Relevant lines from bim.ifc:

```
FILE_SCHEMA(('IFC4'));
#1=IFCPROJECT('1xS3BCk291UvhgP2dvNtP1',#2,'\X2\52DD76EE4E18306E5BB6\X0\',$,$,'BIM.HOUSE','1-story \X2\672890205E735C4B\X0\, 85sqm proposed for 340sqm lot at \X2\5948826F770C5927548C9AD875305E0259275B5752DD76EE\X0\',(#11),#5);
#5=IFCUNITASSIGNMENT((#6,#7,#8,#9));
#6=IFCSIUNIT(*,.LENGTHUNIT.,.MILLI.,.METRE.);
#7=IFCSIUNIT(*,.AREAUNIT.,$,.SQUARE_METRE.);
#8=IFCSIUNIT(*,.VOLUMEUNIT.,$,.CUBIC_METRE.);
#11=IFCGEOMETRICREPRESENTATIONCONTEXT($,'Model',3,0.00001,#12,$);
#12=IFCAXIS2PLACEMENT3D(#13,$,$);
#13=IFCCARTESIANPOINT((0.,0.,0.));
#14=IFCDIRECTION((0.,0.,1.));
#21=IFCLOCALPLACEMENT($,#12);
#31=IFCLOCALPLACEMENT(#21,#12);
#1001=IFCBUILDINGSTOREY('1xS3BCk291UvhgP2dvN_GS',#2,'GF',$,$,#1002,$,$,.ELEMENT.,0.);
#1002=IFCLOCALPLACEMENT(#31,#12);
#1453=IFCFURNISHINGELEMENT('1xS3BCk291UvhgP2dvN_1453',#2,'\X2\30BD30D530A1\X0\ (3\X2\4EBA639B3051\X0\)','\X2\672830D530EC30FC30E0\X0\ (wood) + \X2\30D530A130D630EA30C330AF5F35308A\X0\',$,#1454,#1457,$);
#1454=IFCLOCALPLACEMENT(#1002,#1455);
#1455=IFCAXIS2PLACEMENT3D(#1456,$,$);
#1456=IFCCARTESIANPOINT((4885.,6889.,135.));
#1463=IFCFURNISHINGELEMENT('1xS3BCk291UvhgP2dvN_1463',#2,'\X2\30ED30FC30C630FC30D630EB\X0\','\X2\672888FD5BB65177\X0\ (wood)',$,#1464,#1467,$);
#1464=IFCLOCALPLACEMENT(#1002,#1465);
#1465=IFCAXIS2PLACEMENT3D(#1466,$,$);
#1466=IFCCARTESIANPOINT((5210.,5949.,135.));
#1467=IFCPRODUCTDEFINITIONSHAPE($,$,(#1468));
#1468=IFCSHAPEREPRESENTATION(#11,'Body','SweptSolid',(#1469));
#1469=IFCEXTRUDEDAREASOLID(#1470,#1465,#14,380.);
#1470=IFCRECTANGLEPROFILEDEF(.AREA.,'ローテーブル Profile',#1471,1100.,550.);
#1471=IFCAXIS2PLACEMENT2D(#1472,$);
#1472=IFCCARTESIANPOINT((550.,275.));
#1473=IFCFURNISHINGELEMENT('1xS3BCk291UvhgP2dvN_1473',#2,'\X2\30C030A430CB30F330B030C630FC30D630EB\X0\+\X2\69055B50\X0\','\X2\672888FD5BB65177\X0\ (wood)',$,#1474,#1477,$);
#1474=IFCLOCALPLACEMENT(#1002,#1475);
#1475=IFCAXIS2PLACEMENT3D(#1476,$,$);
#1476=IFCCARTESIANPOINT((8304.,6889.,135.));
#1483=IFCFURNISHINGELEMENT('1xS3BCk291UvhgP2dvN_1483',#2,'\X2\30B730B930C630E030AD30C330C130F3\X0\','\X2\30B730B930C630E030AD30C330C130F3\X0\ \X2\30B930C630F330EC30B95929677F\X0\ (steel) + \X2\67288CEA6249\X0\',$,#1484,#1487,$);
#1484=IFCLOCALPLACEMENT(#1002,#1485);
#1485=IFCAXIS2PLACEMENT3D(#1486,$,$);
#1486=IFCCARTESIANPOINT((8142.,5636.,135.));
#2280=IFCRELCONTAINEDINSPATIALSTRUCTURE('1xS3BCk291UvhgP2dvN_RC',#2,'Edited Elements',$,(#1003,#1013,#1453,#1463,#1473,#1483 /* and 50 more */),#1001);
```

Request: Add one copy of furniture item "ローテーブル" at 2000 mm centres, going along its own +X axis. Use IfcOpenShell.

```python
import ifcopenshell
import ifcopenshell.api.geometry
import ifcopenshell.api.root
import ifcopenshell.util.element
import ifcopenshell.util.placement
import ifcopenshell.util.unit

model = ifcopenshell.open("bim.ifc")
unit_scale = ifcopenshell.util.unit.calculate_unit_scale(model)


def reuse_history(source, copy):
    """copy_class also copies each property set's owner history, people and application; keep the originals."""
    for rel in copy.IsDefinedBy:
        if rel.is_a("IfcRelDefinesByProperties") and (history := rel.RelatingPropertyDefinition.OwnerHistory):
            rel.RelatingPropertyDefinition.OwnerHistory = source.OwnerHistory
            ifcopenshell.util.element.remove_deep2(model, history)


source = model.by_guid("1xS3BCk291UvhgP2dvN_1463")
base = ifcopenshell.util.placement.get_local_placement(source.ObjectPlacement)
step = base[:3, 0] * 2 / unit_scale

for i in range(1, 2):
    copy = ifcopenshell.api.root.copy_class(model, product=source)
    copy.Representation = ifcopenshell.util.element.copy_deep(
        model, source.Representation, exclude=["IfcGeometricRepresentationContext", "IfcRepresentationMap"]
    )
    reuse_history(source, copy)
    matrix = base.copy()
    matrix[:3, 3] += i * step
    print("added at", matrix[:3, 3].round(3) + 0.0)
    ifcopenshell.api.geometry.edit_object_placement(model, product=copy, matrix=matrix, is_si=False)

model.write("bim_edited.ifc")
```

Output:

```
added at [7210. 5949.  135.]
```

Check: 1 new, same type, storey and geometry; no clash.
